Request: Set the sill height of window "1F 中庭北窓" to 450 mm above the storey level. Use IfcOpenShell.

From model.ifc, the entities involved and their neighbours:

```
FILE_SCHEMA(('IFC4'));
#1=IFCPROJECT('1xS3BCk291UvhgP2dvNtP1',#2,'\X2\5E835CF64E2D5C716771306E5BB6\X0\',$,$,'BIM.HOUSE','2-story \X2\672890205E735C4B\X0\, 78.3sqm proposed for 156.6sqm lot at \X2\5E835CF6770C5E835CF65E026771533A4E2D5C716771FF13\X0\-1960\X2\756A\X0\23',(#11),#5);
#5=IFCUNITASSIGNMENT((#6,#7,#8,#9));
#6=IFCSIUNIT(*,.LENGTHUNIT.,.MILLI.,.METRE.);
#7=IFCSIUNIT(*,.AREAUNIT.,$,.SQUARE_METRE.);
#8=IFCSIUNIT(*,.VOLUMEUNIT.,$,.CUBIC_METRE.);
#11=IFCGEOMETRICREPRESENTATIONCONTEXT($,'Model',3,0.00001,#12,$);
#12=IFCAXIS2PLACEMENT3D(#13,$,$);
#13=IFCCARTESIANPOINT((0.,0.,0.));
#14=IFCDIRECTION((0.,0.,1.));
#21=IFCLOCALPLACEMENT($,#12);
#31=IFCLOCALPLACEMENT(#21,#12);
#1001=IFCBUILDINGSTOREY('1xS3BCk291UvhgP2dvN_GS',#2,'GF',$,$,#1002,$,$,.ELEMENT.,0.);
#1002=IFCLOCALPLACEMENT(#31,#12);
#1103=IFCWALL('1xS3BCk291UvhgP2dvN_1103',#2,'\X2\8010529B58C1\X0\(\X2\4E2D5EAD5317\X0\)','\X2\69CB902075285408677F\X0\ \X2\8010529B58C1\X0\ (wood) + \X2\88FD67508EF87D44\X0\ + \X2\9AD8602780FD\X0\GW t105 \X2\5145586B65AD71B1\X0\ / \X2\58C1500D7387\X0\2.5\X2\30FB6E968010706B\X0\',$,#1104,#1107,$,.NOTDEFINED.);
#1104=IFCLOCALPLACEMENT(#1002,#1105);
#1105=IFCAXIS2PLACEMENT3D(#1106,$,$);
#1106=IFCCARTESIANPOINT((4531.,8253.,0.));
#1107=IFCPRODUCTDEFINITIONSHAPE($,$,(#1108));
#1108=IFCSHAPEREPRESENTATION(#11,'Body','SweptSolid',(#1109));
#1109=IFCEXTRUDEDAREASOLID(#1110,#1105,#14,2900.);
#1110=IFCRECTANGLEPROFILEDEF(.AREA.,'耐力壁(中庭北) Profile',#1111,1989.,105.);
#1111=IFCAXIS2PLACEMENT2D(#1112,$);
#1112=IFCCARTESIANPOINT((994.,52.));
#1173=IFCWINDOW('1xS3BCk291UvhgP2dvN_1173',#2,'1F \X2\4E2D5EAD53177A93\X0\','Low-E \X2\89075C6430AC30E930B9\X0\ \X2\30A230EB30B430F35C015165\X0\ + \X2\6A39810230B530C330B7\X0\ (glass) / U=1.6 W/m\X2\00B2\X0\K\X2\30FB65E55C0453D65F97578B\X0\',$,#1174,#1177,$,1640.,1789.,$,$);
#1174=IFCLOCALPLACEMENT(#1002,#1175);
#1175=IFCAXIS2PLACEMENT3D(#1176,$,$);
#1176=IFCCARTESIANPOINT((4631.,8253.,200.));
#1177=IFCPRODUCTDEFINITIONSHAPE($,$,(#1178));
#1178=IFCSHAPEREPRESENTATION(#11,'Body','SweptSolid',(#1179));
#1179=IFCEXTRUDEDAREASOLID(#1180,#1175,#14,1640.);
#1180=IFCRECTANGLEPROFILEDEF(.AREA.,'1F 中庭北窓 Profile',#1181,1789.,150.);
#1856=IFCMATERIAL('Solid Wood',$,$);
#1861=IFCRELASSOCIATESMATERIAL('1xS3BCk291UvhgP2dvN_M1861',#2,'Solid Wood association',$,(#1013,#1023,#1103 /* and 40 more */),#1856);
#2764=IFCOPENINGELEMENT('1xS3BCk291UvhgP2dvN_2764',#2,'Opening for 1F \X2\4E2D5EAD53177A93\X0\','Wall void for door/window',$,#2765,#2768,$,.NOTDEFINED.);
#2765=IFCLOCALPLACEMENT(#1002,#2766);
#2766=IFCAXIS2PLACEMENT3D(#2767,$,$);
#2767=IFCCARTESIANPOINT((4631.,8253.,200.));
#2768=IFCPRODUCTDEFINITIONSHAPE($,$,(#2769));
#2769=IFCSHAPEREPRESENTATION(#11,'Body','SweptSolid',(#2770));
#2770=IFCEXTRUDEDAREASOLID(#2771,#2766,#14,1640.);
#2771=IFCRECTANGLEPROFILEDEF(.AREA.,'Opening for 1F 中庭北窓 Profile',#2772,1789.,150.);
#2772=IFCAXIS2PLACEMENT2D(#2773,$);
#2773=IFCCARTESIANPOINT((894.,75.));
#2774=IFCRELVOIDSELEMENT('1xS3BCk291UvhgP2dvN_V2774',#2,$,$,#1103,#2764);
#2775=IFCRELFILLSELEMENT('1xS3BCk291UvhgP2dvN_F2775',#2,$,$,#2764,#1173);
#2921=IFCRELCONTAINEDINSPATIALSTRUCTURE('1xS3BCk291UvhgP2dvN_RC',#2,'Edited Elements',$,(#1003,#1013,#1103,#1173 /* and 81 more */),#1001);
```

```python
import numpy as np
import ifcopenshell
import ifcopenshell.api.geometry
import ifcopenshell.geom
import ifcopenshell.util.element
import ifcopenshell.util.placement
import ifcopenshell.util.shape
import ifcopenshell.util.unit

model = ifcopenshell.open("model.ifc")
unit_scale = ifcopenshell.util.unit.calculate_unit_scale(model)

window = model.by_id(1173)
opening = window.FillsVoids[0].RelatingOpeningElement
storey = ifcopenshell.util.element.get_container(window, ifc_class="IfcBuildingStorey")
level = ifcopenshell.util.placement.get_local_placement(storey.ObjectPlacement)[2, 3]

# The opening's origin need not be at the sill, so measure its lowest point.
shape = ifcopenshell.geom.create_shape(ifcopenshell.geom.settings(), opening)
bottom = ifcopenshell.util.shape.get_shape_bottom_elevation(shape, shape.geometry) / unit_scale
dz = level + 450.0 - bottom

shift = np.array([0.0, 0.0, dz])
# The window is not placed relative to its opening, so move both.
for product in (opening, window):
    matrix = ifcopenshell.util.placement.get_local_placement(product.ObjectPlacement)
    matrix[:3, 3] += shift
    ifcopenshell.api.geometry.edit_object_placement(model, product=product, matrix=matrix, is_si=False)

print(f"moved by {dz * unit_scale:+.3f} m")

model.write("model_v2.ifc")
```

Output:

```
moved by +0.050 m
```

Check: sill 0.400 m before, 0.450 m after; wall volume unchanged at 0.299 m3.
